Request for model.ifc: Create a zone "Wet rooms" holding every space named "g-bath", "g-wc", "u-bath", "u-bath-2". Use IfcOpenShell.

First a look at what the model holds.

```python
import ifcopenshell

model = ifcopenshell.open("model.ifc")
print(model.schema)
seen = {}
for space in model.by_type("IfcSpace"):
    seen[space.LongName] = seen.get(space.LongName, 0) + 1
for name, count in sorted(seen.items(), key=str):
    print(count, "x", name)
print("zones:", [z.Name for z in model.by_type("IfcZone")][:20])
```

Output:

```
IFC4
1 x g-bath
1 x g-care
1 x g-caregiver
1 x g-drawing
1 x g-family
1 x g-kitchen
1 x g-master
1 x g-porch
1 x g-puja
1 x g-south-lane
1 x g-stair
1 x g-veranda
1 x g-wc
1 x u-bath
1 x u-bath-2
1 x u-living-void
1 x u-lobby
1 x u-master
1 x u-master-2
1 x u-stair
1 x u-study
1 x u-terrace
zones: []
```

```python
import ifcopenshell
import ifcopenshell.api.group
import ifcopenshell.api.root

model = ifcopenshell.open("model.ifc")

names = {"g-bath", "g-wc", "u-bath", "u-bath-2"}
spaces = [s for s in model.by_type("IfcSpace") if s.LongName in names]

zone = ifcopenshell.api.root.create_entity(model, ifc_class="IfcZone", name="Wet rooms")
ifcopenshell.api.group.assign_group(model, products=spaces, group=zone)
print(len(spaces), "spaces in", zone.Name)

model.write("model_rev.ifc")
```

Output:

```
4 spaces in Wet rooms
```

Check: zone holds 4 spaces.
